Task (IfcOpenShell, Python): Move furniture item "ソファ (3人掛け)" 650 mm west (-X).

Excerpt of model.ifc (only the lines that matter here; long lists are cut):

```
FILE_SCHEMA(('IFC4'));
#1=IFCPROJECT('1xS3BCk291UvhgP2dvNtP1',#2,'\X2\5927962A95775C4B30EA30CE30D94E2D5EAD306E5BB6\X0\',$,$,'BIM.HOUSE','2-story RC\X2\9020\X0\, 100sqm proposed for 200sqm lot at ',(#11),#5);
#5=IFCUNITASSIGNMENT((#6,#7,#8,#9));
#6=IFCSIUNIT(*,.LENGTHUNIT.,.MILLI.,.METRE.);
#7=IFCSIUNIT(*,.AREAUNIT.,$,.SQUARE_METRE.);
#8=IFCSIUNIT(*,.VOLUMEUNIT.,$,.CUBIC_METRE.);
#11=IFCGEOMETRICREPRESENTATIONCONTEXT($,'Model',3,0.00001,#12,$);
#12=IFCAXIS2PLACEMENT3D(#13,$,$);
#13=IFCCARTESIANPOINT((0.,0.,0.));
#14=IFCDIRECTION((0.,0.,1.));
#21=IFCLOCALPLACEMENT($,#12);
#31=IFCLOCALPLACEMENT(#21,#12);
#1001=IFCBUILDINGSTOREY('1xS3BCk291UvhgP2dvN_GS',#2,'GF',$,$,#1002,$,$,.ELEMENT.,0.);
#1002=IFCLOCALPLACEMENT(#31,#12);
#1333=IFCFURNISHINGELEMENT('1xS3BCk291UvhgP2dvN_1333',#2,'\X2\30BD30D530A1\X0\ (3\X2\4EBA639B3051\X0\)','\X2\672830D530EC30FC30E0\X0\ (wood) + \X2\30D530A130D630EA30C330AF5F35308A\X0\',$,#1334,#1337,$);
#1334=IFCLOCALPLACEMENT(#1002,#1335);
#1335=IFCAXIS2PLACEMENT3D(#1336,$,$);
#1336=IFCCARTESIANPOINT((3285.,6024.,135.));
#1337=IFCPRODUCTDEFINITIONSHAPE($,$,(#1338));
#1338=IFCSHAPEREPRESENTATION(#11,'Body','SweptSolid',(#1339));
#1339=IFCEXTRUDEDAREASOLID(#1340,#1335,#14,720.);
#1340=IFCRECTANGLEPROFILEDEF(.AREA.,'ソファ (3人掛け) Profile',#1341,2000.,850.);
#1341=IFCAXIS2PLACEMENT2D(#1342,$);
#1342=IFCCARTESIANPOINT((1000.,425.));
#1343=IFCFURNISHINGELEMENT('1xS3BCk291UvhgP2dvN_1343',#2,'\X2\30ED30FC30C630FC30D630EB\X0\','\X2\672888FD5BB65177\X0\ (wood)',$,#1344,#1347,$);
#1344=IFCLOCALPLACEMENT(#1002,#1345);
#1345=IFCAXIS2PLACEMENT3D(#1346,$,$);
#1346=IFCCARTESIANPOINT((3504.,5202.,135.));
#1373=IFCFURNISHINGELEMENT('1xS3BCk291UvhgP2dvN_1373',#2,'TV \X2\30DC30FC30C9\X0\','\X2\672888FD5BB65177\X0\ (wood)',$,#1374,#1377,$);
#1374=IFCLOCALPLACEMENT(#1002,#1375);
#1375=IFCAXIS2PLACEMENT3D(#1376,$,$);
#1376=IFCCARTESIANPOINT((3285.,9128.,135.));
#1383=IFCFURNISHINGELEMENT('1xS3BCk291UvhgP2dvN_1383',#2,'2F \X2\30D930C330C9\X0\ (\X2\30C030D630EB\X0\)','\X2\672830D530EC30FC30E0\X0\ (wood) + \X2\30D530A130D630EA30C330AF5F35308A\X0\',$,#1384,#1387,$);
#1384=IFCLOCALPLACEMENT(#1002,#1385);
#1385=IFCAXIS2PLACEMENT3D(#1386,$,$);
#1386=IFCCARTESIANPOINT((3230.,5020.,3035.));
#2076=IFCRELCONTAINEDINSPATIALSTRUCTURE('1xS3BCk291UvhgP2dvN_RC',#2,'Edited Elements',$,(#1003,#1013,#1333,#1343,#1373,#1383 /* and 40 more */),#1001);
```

```python
import ifcopenshell
import ifcopenshell.api.geometry
import ifcopenshell.util.placement
import ifcopenshell.util.unit

model = ifcopenshell.open("model.ifc")
unit_scale = ifcopenshell.util.unit.calculate_unit_scale(model)

item = model.by_id(1333)
matrix = ifcopenshell.util.placement.get_local_placement(item.ObjectPlacement)
matrix[0, 3] -= 0.65 / unit_scale
ifcopenshell.api.geometry.edit_object_placement(model, product=item, matrix=matrix, is_si=False)

print(ifcopenshell.util.placement.get_local_placement(item.ObjectPlacement).round(3) + 0.0)

model.write("model_updated.ifc")
```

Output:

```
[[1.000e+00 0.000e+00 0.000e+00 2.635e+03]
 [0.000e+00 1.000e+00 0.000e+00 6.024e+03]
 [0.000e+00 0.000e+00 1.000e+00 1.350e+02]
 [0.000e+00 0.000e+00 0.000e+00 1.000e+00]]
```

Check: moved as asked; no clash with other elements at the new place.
